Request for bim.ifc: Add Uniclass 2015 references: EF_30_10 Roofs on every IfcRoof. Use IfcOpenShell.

First a look at what the model holds.

```python
import ifcopenshell

model = ifcopenshell.open("bim.ifc")
print(model.schema)
print("classifications:", [c.Name for c in model.by_type("IfcClassification")])
for ifc_class in ("IfcDoor", "IfcRoof", "IfcStair", "IfcWall", "IfcWindow"):
    print(ifc_class, len(model.by_type(ifc_class)))
```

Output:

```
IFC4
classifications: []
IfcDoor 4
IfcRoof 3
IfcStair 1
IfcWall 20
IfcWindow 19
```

```python
import ifcopenshell
import ifcopenshell.api.classification

model = ifcopenshell.open("bim.ifc")

system = ifcopenshell.api.classification.add_classification(model, classification="Uniclass 2015")

codes = {
    "IfcRoof": ("EF_30_10", "Roofs"),
}
for ifc_class, (code, name) in codes.items():
    products = model.by_type(ifc_class)
    ifcopenshell.api.classification.add_reference(
        model, products=products, classification=system, identification=code, name=name
    )
    print(code, len(products))

model.write("bim_edited.ifc")
```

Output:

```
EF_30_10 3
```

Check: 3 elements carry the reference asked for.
